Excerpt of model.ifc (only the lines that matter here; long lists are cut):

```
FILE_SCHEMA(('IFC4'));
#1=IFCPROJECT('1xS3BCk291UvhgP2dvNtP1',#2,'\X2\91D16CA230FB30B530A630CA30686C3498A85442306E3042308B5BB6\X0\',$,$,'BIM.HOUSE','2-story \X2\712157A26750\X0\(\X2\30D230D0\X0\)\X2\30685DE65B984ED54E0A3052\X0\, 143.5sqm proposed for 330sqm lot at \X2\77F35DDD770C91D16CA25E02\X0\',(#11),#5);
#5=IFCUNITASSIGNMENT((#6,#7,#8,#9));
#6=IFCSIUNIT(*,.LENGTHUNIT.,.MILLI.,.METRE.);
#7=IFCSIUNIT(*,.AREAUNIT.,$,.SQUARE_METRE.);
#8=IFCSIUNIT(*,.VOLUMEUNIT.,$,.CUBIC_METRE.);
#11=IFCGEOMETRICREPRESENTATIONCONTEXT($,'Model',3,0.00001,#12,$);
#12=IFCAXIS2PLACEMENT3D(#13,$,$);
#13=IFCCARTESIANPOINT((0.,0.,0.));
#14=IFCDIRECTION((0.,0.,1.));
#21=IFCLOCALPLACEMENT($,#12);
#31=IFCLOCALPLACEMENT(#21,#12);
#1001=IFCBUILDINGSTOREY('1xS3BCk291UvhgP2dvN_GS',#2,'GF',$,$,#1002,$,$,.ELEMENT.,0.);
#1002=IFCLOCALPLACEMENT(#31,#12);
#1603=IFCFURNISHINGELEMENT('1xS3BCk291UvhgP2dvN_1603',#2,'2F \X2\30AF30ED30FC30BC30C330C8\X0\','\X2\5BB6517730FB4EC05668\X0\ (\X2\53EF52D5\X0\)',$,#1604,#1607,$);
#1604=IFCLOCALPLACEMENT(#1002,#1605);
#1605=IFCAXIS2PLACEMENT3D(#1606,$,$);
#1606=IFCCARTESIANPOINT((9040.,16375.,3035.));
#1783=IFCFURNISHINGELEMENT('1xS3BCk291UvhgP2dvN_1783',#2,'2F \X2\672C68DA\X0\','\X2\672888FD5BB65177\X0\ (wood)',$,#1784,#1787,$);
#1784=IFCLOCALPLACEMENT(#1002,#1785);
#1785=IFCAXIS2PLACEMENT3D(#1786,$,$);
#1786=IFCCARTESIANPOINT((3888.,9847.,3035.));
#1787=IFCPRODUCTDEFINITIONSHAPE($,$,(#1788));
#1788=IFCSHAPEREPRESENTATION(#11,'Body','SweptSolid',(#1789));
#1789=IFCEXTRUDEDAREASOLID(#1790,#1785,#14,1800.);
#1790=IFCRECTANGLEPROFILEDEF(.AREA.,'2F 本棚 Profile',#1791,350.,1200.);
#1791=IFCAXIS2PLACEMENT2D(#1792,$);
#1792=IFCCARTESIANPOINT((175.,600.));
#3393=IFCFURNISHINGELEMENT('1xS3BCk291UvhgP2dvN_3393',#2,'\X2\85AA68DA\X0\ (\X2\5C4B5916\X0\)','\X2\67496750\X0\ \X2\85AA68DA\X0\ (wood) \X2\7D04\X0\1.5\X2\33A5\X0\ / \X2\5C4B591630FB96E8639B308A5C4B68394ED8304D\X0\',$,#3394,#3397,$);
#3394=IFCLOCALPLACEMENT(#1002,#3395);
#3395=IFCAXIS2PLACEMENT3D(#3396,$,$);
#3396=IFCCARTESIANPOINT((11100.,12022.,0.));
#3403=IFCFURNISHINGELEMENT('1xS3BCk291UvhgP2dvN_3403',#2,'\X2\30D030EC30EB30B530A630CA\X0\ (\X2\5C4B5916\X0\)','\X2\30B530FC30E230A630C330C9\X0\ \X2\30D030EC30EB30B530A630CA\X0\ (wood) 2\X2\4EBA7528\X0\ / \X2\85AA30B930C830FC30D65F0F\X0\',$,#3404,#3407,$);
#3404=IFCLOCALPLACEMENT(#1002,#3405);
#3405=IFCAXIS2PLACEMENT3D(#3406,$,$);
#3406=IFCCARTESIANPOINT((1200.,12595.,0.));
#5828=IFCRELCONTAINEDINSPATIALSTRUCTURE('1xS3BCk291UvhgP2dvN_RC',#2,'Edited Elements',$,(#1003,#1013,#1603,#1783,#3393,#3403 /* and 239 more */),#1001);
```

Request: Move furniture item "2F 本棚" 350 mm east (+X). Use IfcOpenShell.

```python
import ifcopenshell
import ifcopenshell.api.geometry
import ifcopenshell.util.placement
import ifcopenshell.util.unit

model = ifcopenshell.open("model.ifc")
unit_scale = ifcopenshell.util.unit.calculate_unit_scale(model)

item = model.by_guid("1xS3BCk291UvhgP2dvN_1783")
matrix = ifcopenshell.util.placement.get_local_placement(item.ObjectPlacement)
matrix[0, 3] += 0.35 / unit_scale
ifcopenshell.api.geometry.edit_object_placement(model, product=item, matrix=matrix, is_si=False)

print(ifcopenshell.util.placement.get_local_placement(item.ObjectPlacement).round(3) + 0.0)

model.write("model_edited.ifc")
```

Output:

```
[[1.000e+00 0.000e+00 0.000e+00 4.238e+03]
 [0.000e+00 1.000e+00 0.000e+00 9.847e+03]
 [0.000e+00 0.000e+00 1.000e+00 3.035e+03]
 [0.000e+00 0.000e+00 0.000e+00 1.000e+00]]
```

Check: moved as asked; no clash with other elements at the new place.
